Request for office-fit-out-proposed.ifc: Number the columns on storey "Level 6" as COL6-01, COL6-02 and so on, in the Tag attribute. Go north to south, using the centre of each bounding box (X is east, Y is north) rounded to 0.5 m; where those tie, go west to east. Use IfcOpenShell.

First a look at what the model holds.

```python
import ifcopenshell
import ifcopenshell.util.element
import ifcopenshell.util.placement

model = ifcopenshell.open("office-fit-out-proposed.ifc")
print(model.schema)
storey = next(s for s in model.by_type("IfcBuildingStorey") if s.Name == "Level 6")
columns = [e for e in ifcopenshell.util.element.get_decomposition(storey) if e.is_a("IfcColumn")]
for e in sorted(columns, key=lambda e: e.id()):
    origin = ifcopenshell.util.placement.get_local_placement(e.ObjectPlacement)[:3, 3]
    print(e.id(), e.Tag, e.Name, origin.round(2) + 0.0, sep=" | ")
```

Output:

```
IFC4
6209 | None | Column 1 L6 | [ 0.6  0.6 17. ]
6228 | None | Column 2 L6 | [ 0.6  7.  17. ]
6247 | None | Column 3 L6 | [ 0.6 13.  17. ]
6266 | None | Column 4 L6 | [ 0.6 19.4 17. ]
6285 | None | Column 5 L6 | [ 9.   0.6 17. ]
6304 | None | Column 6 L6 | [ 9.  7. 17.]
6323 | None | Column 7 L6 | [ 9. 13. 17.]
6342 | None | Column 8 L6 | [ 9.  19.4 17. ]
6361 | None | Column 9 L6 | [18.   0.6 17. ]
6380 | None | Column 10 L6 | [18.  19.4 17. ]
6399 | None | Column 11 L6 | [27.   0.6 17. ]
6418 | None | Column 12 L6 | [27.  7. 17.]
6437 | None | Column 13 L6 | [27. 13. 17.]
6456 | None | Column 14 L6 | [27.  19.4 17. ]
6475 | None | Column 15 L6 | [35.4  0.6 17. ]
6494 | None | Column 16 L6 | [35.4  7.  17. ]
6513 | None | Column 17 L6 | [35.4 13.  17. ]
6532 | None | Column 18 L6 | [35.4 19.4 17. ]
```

```python
import ifcopenshell
import ifcopenshell.geom
import ifcopenshell.util.element
import ifcopenshell.util.shape

model = ifcopenshell.open("office-fit-out-proposed.ifc")
settings = ifcopenshell.geom.settings()
settings.set("use-world-coords", True)


def centre(element):
    shape = ifcopenshell.geom.create_shape(settings, element)
    return ifcopenshell.util.shape.get_bbox_centroid(shape.geometry)


storey = next(s for s in model.by_type("IfcBuildingStorey") if s.Name == "Level 6")
columns = [e for e in ifcopenshell.util.element.get_decomposition(storey) if e.is_a("IfcColumn")]

# Insertion points can sit at a corner or the storey origin, so sort by the geometry (in metres).
centres = {e: centre(e) for e in columns}
columns.sort(key=lambda e: (-round(centres[e][1] / 0.5), centres[e][0]))

for i, e in enumerate(columns, start=1):
    number = f"COL6-{i:02d}"
    e.Tag = number
    print(e.id(), number)

model.write("office-fit-out-proposed-out.ifc")
```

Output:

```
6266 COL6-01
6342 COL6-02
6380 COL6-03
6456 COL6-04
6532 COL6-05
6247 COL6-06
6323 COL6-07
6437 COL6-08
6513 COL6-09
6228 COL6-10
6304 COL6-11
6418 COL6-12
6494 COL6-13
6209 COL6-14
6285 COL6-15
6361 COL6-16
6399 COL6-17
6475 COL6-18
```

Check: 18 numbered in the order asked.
